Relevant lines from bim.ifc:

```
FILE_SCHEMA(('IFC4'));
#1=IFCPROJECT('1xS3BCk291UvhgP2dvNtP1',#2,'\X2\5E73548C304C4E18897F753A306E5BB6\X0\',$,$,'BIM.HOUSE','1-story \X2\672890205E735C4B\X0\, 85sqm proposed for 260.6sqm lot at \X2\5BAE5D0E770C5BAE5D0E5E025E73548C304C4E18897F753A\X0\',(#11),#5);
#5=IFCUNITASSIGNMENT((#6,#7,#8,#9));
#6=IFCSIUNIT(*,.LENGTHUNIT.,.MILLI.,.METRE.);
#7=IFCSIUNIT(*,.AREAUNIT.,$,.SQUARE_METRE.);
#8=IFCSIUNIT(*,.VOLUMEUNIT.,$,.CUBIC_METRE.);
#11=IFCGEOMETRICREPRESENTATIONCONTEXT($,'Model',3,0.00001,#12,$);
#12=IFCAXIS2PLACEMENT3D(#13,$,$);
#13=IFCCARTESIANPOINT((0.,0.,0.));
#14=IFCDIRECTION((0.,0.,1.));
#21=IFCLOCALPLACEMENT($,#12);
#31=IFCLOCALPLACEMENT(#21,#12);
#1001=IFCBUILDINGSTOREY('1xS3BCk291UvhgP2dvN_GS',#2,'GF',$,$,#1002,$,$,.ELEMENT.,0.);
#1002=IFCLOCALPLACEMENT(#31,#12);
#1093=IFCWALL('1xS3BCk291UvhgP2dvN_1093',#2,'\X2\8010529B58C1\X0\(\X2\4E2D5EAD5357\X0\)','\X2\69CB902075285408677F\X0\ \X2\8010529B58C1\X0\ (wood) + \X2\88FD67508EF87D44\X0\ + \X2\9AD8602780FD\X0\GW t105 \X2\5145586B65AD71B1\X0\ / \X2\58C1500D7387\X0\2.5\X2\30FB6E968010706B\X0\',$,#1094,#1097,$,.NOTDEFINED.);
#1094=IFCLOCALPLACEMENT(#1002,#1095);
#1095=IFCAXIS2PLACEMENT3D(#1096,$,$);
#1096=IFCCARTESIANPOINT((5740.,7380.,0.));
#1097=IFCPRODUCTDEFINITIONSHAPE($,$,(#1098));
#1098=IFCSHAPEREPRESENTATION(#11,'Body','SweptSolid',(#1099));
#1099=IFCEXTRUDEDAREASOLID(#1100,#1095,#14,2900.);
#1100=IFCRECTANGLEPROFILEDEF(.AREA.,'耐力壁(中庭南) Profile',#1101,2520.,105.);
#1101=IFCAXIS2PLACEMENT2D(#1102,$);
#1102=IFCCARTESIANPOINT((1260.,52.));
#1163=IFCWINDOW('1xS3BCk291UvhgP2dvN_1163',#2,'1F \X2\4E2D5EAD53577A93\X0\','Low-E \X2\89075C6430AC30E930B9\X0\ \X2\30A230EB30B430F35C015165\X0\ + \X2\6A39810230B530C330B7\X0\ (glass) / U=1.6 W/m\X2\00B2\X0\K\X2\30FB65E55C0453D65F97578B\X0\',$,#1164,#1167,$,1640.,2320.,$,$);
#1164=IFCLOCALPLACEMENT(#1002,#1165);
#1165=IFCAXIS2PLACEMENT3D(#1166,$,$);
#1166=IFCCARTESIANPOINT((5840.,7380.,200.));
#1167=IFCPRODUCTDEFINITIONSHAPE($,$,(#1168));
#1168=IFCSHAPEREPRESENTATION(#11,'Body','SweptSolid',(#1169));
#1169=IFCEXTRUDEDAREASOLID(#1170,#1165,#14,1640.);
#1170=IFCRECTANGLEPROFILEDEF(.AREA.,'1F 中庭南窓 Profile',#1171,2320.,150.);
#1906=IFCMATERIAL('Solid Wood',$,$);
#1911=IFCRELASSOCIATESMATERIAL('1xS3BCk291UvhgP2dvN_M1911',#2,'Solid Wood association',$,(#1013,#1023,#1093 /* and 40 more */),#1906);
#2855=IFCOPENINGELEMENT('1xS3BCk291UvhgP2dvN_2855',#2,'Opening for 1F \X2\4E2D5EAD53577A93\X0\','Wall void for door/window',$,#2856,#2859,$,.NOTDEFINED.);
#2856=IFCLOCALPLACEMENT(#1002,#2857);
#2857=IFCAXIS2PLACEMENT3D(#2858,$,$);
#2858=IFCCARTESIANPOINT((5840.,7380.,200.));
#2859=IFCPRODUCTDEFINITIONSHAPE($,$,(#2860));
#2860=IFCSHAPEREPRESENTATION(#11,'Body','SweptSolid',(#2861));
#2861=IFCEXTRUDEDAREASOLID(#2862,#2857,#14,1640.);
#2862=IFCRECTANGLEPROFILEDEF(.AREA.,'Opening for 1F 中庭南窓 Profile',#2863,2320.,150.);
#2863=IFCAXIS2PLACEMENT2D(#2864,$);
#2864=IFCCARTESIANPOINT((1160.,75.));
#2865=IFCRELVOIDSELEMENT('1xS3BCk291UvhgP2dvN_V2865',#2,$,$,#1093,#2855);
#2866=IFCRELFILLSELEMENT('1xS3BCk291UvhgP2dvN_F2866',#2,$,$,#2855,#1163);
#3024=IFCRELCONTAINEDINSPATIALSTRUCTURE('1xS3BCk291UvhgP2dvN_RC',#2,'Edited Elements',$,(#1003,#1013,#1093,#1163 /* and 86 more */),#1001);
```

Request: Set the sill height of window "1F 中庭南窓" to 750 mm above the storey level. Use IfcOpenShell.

```python
import numpy as np
import ifcopenshell
import ifcopenshell.api.geometry
import ifcopenshell.geom
import ifcopenshell.util.element
import ifcopenshell.util.placement
import ifcopenshell.util.shape
import ifcopenshell.util.unit

model = ifcopenshell.open("bim.ifc")
unit_scale = ifcopenshell.util.unit.calculate_unit_scale(model)

window = model.by_guid("1xS3BCk291UvhgP2dvN_1163")
opening = window.FillsVoids[0].RelatingOpeningElement
storey = ifcopenshell.util.element.get_container(window, ifc_class="IfcBuildingStorey")
level = ifcopenshell.util.placement.get_local_placement(storey.ObjectPlacement)[2, 3]

# The opening's origin need not be at the sill, so measure its lowest point.
shape = ifcopenshell.geom.create_shape(ifcopenshell.geom.settings(), opening)
bottom = ifcopenshell.util.shape.get_shape_bottom_elevation(shape, shape.geometry) / unit_scale
dz = level + 0.75 / unit_scale - bottom

shift = np.array([0.0, 0.0, dz])
# The window is not placed relative to its opening, so move both.
for product in (opening, window):
    matrix = ifcopenshell.util.placement.get_local_placement(product.ObjectPlacement)
    matrix[:3, 3] += shift
    ifcopenshell.api.geometry.edit_object_placement(model, product=product, matrix=matrix, is_si=False)

print(f"moved by {dz * unit_scale:+.3f} m")

model.write("bim_rev.ifc")
```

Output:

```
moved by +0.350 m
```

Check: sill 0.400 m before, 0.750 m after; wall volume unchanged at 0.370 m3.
